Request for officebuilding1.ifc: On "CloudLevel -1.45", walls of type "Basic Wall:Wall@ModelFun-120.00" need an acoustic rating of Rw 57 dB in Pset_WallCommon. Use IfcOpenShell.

First a look at what the model holds.

```python
import ifcopenshell
import ifcopenshell.util.element

model = ifcopenshell.open("officebuilding1.ifc")
print(model.schema)
storey = next(s for s in model.by_type("IfcBuildingStorey") if s.Name == "CloudLevel -1.45")
walls = [e for e in ifcopenshell.util.element.get_decomposition(storey) if e.is_a("IfcWall")]
seen = {}
for e in walls:
    element_type = ifcopenshell.util.element.get_type(e)
    key = (element_type.Name if element_type != e and element_type else None, ifcopenshell.util.element.get_pset(e, "Pset_WallCommon", "AcousticRating"))
    seen[key] = seen.get(key, 0) + 1
for (name, value), count in sorted(seen.items(), key=str):
    print(count, "x", name, "|", value)
```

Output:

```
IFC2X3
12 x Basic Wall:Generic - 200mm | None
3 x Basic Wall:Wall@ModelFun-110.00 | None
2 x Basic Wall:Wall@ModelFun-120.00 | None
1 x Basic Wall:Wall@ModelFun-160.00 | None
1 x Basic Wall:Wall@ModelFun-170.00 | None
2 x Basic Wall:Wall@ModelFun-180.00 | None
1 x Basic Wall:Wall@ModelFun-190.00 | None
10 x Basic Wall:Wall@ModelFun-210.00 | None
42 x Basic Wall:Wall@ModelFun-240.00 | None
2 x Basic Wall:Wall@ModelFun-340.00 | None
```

```python
import ifcopenshell
import ifcopenshell.api.pset
import ifcopenshell.util.element

model = ifcopenshell.open("officebuilding1.ifc")

storey = next(s for s in model.by_type("IfcBuildingStorey") if s.Name == "CloudLevel -1.45")
walls = [e for e in ifcopenshell.util.element.get_decomposition(storey) if e.is_a("IfcWall")]

count = 0
for e in walls:
    element_type = ifcopenshell.util.element.get_type(e)
    if element_type in (None, e) or element_type.Name != "Basic Wall:Wall@ModelFun-120.00":
        continue
    # add_pset returns the element's existing set when there is one.
    pset = ifcopenshell.api.pset.add_pset(model, product=e, name="Pset_WallCommon")
    ifcopenshell.api.pset.edit_pset(model, pset=pset, properties={"AcousticRating": "Rw 57 dB"})
    count += 1

print(count, "walls updated")

model.write("officebuilding1_edited.ifc")
```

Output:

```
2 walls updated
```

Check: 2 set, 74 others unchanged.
